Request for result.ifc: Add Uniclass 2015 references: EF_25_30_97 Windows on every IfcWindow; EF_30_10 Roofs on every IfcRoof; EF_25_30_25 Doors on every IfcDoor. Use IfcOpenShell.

First a look at what the model holds.

```python
import ifcopenshell

model = ifcopenshell.open("result.ifc")
print(model.schema)
print("classifications:", [c.Name for c in model.by_type("IfcClassification")])
for ifc_class in ("IfcDoor", "IfcRoof", "IfcStair", "IfcWall", "IfcWindow"):
    print(ifc_class, len(model.by_type(ifc_class)))
```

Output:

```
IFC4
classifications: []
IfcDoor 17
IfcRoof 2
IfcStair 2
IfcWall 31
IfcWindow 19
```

```python
import ifcopenshell
import ifcopenshell.api.classification

model = ifcopenshell.open("result.ifc")

system = ifcopenshell.api.classification.add_classification(model, classification="Uniclass 2015")

codes = {
    "IfcWindow": ("EF_25_30_97", "Windows"),
    "IfcRoof": ("EF_30_10", "Roofs"),
    "IfcDoor": ("EF_25_30_25", "Doors"),
}
for ifc_class, (code, name) in codes.items():
    products = model.by_type(ifc_class)
    ifcopenshell.api.classification.add_reference(
        model, products=products, classification=system, identification=code, name=name
    )
    print(code, len(products))

model.write("result_v2.ifc")
```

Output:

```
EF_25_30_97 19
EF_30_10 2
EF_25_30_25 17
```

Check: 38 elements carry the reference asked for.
